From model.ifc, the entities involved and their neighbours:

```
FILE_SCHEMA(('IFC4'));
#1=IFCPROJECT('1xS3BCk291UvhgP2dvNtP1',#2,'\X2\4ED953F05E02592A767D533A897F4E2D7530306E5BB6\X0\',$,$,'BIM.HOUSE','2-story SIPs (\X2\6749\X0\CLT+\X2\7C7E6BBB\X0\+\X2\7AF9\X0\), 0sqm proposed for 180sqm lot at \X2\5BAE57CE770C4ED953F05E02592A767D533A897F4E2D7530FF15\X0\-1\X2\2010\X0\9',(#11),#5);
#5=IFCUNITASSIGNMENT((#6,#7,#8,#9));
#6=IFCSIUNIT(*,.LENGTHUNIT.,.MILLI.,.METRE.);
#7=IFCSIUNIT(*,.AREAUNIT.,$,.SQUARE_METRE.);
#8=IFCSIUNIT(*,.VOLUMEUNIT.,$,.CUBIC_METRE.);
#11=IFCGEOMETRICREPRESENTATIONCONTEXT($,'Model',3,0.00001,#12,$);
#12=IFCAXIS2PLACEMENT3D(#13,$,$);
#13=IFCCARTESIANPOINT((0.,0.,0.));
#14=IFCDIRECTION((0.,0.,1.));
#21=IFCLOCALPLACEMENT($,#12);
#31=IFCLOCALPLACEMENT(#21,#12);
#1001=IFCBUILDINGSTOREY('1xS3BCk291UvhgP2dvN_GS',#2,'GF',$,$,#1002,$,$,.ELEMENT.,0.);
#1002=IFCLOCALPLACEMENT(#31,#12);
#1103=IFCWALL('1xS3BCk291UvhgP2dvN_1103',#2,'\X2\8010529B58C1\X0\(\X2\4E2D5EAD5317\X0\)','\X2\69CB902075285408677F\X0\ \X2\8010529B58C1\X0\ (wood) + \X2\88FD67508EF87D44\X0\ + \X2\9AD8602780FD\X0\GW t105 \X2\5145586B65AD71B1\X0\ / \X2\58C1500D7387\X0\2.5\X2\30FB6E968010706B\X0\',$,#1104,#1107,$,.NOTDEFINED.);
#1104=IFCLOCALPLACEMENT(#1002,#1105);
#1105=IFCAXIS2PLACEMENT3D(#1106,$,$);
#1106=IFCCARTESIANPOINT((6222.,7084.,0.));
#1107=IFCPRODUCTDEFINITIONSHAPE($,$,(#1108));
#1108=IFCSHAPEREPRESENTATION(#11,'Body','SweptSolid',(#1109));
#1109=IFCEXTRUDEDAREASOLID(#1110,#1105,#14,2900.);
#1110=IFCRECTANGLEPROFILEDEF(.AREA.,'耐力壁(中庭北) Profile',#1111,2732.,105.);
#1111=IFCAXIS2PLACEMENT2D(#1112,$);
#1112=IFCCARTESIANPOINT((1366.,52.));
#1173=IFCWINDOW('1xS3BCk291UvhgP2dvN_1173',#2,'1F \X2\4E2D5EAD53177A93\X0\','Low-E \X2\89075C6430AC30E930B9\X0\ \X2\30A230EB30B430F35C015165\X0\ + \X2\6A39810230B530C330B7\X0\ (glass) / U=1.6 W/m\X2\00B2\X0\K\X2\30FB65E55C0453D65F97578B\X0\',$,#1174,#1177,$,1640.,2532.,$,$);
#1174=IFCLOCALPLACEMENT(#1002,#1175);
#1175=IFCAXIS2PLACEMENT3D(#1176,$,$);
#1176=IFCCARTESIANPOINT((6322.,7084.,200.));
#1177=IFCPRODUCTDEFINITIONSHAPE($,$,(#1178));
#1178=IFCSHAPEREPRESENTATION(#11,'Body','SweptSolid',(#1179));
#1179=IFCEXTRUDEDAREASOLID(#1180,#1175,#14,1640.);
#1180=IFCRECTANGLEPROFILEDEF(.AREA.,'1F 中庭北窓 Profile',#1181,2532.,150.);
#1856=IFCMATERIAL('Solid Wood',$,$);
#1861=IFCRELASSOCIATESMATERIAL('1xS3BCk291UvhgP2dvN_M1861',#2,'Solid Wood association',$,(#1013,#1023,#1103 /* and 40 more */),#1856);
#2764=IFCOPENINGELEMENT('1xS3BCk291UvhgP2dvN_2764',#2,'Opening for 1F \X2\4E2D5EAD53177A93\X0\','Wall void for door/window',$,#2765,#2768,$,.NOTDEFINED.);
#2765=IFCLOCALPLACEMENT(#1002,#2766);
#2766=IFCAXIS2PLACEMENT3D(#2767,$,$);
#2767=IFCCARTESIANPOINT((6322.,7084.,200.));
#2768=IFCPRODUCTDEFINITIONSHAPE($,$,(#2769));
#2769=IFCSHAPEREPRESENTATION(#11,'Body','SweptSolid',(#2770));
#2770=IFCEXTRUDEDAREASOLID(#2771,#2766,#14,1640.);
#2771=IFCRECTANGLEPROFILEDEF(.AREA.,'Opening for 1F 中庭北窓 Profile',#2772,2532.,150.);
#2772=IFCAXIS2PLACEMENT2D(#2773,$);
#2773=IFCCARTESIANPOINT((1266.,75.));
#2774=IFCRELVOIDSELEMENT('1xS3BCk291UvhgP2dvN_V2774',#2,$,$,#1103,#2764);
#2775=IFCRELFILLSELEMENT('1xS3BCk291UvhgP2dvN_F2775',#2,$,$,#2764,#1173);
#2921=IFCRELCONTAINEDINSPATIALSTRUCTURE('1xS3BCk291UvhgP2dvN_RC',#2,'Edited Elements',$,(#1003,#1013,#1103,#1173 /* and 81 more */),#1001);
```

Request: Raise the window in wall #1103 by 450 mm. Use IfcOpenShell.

```python
import numpy as np
import ifcopenshell
import ifcopenshell.api.geometry
import ifcopenshell.util.placement
import ifcopenshell.util.unit

model = ifcopenshell.open("model.ifc")
unit_scale = ifcopenshell.util.unit.calculate_unit_scale(model)

window = model.by_id(1173)
opening = window.FillsVoids[0].RelatingOpeningElement
dz = 450.0

shift = np.array([0.0, 0.0, dz])
# The window is not placed relative to its opening, so move both.
for product in (opening, window):
    matrix = ifcopenshell.util.placement.get_local_placement(product.ObjectPlacement)
    matrix[:3, 3] += shift
    ifcopenshell.api.geometry.edit_object_placement(model, product=product, matrix=matrix, is_si=False)

print(f"moved by {dz * unit_scale:+.3f} m")

model.write("model_rev.ifc")
```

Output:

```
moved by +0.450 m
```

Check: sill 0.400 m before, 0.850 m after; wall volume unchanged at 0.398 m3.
